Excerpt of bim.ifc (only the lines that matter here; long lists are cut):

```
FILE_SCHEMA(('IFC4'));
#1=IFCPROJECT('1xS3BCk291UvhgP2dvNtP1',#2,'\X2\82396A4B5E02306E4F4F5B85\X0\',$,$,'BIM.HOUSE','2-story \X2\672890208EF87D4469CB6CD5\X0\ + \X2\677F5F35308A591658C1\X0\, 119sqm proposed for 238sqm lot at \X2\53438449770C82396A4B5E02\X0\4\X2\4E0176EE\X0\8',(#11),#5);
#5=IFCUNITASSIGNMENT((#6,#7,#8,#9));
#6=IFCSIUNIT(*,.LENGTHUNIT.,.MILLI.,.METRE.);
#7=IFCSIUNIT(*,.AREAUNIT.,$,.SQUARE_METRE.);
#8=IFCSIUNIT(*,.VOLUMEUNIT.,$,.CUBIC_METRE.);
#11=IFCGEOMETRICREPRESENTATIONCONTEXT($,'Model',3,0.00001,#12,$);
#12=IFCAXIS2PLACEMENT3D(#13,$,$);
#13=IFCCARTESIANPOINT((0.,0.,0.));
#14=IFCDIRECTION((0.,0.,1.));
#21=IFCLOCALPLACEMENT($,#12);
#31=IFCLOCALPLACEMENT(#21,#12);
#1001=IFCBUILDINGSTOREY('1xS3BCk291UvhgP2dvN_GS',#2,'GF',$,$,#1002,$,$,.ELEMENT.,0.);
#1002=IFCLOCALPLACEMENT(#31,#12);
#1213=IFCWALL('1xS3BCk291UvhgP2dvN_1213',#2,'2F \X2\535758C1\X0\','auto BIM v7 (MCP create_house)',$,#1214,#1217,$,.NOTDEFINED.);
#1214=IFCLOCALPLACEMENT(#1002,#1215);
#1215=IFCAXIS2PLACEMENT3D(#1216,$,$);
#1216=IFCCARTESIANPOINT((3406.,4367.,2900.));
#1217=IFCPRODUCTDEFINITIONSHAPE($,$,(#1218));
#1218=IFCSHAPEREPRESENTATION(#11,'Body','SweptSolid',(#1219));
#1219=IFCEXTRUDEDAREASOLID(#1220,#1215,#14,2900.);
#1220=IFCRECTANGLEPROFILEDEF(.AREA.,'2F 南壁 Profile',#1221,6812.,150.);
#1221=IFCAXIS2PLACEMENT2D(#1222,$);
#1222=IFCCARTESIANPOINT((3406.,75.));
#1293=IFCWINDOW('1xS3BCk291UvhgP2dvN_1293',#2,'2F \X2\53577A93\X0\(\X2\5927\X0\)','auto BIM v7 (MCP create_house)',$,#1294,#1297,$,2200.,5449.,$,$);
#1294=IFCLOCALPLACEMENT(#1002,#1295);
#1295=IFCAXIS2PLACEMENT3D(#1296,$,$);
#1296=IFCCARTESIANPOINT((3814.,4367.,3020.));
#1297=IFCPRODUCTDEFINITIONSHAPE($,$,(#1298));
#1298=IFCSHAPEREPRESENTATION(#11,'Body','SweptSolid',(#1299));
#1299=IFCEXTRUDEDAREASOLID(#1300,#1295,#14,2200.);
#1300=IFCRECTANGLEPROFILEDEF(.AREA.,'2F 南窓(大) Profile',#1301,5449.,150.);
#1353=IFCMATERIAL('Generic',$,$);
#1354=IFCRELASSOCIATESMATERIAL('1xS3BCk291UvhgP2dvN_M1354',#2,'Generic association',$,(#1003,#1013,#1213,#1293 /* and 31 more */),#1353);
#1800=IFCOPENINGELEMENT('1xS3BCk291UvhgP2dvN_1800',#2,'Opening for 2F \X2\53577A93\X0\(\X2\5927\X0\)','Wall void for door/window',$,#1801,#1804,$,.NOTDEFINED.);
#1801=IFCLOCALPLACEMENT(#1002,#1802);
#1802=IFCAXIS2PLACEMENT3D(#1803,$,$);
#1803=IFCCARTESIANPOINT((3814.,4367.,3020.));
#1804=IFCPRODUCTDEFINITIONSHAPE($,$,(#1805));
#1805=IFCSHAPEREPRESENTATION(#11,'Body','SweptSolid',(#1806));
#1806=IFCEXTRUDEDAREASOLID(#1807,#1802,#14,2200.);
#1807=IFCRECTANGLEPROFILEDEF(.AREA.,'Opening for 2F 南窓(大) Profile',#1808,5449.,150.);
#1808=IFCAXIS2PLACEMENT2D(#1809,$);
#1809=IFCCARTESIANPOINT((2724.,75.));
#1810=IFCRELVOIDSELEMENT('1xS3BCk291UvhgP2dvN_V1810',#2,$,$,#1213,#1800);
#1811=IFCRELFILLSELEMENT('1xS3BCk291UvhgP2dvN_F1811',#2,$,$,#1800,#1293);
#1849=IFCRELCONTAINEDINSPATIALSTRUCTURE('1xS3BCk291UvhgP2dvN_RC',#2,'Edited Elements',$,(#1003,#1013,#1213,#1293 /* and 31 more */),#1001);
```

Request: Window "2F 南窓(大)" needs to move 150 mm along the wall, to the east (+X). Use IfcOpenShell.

```python
import ifcopenshell
import ifcopenshell.api.geometry
import ifcopenshell.util.placement
import ifcopenshell.util.unit

model = ifcopenshell.open("bim.ifc")
unit_scale = ifcopenshell.util.unit.calculate_unit_scale(model)

window = model.by_id(1293)
opening = window.FillsVoids[0].RelatingOpeningElement
wall = opening.VoidsElements[0].RelatingBuildingElement

wall_matrix = ifcopenshell.util.placement.get_local_placement(wall.ObjectPlacement)
shift = wall_matrix[:3, 0] * 0.15 / unit_scale
before = ifcopenshell.util.placement.get_local_placement(window.ObjectPlacement)[:3, 3].copy()

# The window is not placed relative to its opening, so move both.
for product in (opening, window):
    matrix = ifcopenshell.util.placement.get_local_placement(product.ObjectPlacement)
    matrix[:3, 3] += shift
    ifcopenshell.api.geometry.edit_object_placement(model, product=product, matrix=matrix, is_si=False)

after = ifcopenshell.util.placement.get_local_placement(window.ObjectPlacement)[:3, 3]
print("window moved by", (after - before).round(3) + 0.0)

model.write("bim_rev.ifc")
```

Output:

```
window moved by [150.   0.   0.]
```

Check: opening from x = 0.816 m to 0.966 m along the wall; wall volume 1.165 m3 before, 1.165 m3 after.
